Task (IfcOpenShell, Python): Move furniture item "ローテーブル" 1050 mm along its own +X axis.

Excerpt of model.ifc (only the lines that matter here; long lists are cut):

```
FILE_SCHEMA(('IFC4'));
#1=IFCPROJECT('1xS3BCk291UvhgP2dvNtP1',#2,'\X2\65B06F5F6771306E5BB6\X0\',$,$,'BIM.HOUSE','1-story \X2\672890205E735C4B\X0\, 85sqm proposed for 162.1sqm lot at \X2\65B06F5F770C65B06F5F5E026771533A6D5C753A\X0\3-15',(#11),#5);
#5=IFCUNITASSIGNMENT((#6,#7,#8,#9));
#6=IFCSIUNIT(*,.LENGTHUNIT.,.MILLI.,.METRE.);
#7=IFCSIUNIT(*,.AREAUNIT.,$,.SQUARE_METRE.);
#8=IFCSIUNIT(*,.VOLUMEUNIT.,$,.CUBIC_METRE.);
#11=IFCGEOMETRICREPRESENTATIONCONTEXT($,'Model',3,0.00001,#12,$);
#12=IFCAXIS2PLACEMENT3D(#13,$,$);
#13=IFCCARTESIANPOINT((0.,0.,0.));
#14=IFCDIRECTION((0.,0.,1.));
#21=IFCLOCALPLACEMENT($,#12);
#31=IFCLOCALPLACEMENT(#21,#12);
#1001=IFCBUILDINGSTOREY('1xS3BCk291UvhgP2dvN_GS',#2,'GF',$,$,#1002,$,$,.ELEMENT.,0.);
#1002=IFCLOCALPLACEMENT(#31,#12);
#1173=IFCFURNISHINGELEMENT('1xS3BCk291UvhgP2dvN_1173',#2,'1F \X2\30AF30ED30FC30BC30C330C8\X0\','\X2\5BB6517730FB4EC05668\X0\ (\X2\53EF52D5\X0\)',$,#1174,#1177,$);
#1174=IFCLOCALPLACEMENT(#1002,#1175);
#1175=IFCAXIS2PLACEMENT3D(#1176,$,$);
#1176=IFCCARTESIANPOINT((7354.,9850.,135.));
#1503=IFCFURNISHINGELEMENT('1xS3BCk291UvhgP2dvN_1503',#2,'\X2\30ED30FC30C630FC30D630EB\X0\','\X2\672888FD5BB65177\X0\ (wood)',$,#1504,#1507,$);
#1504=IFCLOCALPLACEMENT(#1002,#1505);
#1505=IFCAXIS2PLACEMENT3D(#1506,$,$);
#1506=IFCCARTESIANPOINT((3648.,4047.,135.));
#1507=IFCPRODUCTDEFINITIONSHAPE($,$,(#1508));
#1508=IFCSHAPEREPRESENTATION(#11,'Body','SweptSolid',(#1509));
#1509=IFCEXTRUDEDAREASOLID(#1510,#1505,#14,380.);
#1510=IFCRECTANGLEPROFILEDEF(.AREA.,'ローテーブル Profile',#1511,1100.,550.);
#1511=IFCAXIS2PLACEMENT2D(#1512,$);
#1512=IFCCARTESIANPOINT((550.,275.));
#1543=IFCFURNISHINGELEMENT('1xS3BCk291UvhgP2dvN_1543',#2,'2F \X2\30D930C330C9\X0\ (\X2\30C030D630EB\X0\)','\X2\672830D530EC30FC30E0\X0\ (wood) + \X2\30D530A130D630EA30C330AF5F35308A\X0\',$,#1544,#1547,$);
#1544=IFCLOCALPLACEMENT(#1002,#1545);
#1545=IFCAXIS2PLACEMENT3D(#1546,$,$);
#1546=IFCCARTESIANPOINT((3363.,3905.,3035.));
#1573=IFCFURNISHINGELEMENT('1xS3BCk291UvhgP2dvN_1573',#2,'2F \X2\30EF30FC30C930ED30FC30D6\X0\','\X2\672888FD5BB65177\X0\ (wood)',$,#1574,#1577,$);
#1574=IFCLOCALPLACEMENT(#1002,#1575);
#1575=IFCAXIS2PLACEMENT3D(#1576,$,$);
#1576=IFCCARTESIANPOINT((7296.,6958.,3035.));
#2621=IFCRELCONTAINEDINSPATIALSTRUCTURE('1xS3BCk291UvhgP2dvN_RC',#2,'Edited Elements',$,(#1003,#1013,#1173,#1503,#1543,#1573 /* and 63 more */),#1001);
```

```python
import ifcopenshell
import ifcopenshell.api.geometry
import ifcopenshell.util.placement
import ifcopenshell.util.unit

model = ifcopenshell.open("model.ifc")
unit_scale = ifcopenshell.util.unit.calculate_unit_scale(model)

item = model.by_guid("1xS3BCk291UvhgP2dvN_1503")
matrix = ifcopenshell.util.placement.get_local_placement(item.ObjectPlacement)
matrix[:3, 3] += matrix[:3, 0] * 1.05 / unit_scale
ifcopenshell.api.geometry.edit_object_placement(model, product=item, matrix=matrix, is_si=False)

print(ifcopenshell.util.placement.get_local_placement(item.ObjectPlacement).round(3) + 0.0)

model.write("model_updated.ifc")
```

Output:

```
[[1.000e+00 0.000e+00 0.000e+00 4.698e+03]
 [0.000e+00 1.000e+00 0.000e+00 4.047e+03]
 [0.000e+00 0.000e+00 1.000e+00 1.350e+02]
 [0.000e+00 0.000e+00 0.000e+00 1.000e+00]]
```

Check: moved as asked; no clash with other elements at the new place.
